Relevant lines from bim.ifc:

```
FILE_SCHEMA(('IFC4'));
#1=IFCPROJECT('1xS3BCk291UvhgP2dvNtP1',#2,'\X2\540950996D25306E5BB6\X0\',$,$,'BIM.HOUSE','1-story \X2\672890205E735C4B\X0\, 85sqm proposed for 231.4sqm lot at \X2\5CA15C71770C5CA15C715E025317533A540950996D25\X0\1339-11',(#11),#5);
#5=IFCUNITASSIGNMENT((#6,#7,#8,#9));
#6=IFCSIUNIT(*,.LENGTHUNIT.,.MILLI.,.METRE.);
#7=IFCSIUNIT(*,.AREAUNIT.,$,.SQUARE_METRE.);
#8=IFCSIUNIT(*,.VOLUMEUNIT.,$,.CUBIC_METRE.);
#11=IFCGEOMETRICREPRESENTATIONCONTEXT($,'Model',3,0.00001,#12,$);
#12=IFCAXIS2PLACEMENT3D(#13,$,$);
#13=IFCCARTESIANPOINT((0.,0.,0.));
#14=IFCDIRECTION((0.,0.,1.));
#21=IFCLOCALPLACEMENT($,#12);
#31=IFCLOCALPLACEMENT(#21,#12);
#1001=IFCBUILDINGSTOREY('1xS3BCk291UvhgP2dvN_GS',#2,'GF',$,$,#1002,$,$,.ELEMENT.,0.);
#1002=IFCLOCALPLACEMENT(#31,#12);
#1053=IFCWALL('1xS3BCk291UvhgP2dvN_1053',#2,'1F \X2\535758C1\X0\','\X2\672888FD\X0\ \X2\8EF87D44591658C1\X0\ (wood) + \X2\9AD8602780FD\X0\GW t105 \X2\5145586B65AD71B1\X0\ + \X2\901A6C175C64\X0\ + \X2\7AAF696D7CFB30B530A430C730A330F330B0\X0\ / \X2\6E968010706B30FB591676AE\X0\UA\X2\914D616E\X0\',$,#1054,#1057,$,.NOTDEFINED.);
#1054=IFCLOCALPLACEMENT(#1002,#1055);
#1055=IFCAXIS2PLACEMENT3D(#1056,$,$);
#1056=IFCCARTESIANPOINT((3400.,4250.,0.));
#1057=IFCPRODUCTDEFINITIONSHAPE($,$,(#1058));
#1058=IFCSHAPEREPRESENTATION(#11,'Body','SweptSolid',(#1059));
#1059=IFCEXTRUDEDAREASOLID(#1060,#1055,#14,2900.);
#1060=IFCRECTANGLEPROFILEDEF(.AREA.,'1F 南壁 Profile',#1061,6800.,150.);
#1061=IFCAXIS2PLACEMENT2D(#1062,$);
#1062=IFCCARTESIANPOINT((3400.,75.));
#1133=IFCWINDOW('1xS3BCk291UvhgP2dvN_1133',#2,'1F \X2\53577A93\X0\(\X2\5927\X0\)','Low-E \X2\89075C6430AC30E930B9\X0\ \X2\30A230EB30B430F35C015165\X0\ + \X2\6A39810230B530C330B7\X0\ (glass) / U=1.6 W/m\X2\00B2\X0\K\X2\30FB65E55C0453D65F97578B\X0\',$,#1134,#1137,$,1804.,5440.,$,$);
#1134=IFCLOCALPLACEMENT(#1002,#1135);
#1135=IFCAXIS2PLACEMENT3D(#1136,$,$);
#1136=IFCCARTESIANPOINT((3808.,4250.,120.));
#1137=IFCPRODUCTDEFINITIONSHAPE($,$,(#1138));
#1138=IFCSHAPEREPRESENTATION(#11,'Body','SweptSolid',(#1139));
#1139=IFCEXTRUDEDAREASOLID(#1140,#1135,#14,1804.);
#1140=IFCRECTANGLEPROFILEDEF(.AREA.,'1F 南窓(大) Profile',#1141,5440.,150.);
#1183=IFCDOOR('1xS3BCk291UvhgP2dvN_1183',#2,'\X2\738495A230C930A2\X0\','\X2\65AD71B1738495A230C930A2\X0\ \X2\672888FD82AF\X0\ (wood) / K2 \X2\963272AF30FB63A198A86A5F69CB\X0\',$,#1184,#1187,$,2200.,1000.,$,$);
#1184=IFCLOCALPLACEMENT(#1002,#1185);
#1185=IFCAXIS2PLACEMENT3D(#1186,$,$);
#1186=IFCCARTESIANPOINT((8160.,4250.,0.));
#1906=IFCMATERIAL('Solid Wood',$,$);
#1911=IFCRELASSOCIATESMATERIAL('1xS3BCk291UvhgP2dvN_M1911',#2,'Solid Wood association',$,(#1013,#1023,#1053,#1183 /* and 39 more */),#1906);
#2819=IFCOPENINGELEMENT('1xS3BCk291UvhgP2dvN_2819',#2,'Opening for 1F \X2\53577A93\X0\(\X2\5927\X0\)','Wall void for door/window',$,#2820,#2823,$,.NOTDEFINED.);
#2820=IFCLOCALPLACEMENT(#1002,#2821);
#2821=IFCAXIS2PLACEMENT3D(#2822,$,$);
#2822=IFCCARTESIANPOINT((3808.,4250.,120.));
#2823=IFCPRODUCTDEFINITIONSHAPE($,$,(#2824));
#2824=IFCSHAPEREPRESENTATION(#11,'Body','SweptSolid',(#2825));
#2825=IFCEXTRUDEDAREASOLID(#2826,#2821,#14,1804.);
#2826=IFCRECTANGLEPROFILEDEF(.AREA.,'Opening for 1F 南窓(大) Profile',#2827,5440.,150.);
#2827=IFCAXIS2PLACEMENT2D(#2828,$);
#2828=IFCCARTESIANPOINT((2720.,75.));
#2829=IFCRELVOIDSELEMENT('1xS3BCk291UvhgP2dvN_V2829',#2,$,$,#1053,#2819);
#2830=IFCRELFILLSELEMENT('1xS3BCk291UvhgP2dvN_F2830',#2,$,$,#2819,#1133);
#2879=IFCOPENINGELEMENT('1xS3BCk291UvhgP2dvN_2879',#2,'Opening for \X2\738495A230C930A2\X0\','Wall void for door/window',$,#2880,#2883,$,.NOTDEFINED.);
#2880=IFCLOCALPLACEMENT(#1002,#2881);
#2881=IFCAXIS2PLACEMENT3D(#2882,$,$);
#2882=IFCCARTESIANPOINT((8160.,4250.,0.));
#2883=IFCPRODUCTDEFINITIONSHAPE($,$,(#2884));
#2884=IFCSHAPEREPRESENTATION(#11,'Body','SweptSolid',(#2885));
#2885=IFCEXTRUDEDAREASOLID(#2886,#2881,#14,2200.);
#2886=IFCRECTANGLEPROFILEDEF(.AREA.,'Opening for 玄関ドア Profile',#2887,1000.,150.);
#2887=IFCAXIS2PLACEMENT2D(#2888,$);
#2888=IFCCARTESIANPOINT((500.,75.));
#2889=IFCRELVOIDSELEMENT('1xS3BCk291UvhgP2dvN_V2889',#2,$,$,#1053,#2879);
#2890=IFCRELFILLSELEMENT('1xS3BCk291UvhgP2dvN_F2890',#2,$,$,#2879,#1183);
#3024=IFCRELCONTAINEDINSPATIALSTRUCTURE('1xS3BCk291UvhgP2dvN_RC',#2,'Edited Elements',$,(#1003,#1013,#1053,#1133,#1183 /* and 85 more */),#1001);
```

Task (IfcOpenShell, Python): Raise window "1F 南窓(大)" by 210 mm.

```python
import numpy as np
import ifcopenshell
import ifcopenshell.api.geometry
import ifcopenshell.util.placement
import ifcopenshell.util.unit

model = ifcopenshell.open("bim.ifc")
unit_scale = ifcopenshell.util.unit.calculate_unit_scale(model)

window = model.by_guid("1xS3BCk291UvhgP2dvN_1133")
opening = window.FillsVoids[0].RelatingOpeningElement
dz = 0.21 / unit_scale

shift = np.array([0.0, 0.0, dz])
# The window is not placed relative to its opening, so move both.
for product in (opening, window):
    matrix = ifcopenshell.util.placement.get_local_placement(product.ObjectPlacement)
    matrix[:3, 3] += shift
    ifcopenshell.api.geometry.edit_object_placement(model, product=product, matrix=matrix, is_si=False)

print(f"moved by {dz * unit_scale:+.3f} m")

model.write("bim_edited.ifc")
```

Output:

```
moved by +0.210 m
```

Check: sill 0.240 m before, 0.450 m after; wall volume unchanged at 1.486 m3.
